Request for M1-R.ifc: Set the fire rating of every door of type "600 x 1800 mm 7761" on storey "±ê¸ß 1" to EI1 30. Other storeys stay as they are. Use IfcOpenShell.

First a look at what the model holds.

```python
import ifcopenshell
import ifcopenshell.util.element

model = ifcopenshell.open("M1-R.ifc")
print(model.schema)
storey = next(s for s in model.by_type("IfcBuildingStorey") if s.Name == "±ê¸ß 1")
doors = [e for e in ifcopenshell.util.element.get_decomposition(storey) if e.is_a("IfcDoor")]
seen = {}
for e in doors:
    element_type = ifcopenshell.util.element.get_type(e)
    key = (element_type.Name if element_type != e and element_type else None, ifcopenshell.util.element.get_pset(e, "Pset_DoorCommon", "FireRating"))
    seen[key] = seen.get(key, 0) + 1
for (name, value), count in sorted(seen.items(), key=str):
    print(count, "x", name, "|", value)
```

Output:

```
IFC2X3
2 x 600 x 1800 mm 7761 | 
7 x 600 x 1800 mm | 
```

```python
import ifcopenshell
import ifcopenshell.api.pset
import ifcopenshell.util.element

model = ifcopenshell.open("M1-R.ifc")

storey = next(s for s in model.by_type("IfcBuildingStorey") if s.Name == "±ê¸ß 1")
doors = [e for e in ifcopenshell.util.element.get_decomposition(storey) if e.is_a("IfcDoor")]

count = 0
for e in doors:
    element_type = ifcopenshell.util.element.get_type(e)
    if element_type in (None, e) or element_type.Name != "600 x 1800 mm 7761":
        continue
    # add_pset returns the element's existing set when there is one.
    pset = ifcopenshell.api.pset.add_pset(model, product=e, name="Pset_DoorCommon")
    ifcopenshell.api.pset.edit_pset(model, pset=pset, properties={"FireRating": "EI1 30"})
    count += 1

print(count, "doors updated")

model.write("M1-R_edited.ifc")
```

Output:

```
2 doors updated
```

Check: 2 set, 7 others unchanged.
